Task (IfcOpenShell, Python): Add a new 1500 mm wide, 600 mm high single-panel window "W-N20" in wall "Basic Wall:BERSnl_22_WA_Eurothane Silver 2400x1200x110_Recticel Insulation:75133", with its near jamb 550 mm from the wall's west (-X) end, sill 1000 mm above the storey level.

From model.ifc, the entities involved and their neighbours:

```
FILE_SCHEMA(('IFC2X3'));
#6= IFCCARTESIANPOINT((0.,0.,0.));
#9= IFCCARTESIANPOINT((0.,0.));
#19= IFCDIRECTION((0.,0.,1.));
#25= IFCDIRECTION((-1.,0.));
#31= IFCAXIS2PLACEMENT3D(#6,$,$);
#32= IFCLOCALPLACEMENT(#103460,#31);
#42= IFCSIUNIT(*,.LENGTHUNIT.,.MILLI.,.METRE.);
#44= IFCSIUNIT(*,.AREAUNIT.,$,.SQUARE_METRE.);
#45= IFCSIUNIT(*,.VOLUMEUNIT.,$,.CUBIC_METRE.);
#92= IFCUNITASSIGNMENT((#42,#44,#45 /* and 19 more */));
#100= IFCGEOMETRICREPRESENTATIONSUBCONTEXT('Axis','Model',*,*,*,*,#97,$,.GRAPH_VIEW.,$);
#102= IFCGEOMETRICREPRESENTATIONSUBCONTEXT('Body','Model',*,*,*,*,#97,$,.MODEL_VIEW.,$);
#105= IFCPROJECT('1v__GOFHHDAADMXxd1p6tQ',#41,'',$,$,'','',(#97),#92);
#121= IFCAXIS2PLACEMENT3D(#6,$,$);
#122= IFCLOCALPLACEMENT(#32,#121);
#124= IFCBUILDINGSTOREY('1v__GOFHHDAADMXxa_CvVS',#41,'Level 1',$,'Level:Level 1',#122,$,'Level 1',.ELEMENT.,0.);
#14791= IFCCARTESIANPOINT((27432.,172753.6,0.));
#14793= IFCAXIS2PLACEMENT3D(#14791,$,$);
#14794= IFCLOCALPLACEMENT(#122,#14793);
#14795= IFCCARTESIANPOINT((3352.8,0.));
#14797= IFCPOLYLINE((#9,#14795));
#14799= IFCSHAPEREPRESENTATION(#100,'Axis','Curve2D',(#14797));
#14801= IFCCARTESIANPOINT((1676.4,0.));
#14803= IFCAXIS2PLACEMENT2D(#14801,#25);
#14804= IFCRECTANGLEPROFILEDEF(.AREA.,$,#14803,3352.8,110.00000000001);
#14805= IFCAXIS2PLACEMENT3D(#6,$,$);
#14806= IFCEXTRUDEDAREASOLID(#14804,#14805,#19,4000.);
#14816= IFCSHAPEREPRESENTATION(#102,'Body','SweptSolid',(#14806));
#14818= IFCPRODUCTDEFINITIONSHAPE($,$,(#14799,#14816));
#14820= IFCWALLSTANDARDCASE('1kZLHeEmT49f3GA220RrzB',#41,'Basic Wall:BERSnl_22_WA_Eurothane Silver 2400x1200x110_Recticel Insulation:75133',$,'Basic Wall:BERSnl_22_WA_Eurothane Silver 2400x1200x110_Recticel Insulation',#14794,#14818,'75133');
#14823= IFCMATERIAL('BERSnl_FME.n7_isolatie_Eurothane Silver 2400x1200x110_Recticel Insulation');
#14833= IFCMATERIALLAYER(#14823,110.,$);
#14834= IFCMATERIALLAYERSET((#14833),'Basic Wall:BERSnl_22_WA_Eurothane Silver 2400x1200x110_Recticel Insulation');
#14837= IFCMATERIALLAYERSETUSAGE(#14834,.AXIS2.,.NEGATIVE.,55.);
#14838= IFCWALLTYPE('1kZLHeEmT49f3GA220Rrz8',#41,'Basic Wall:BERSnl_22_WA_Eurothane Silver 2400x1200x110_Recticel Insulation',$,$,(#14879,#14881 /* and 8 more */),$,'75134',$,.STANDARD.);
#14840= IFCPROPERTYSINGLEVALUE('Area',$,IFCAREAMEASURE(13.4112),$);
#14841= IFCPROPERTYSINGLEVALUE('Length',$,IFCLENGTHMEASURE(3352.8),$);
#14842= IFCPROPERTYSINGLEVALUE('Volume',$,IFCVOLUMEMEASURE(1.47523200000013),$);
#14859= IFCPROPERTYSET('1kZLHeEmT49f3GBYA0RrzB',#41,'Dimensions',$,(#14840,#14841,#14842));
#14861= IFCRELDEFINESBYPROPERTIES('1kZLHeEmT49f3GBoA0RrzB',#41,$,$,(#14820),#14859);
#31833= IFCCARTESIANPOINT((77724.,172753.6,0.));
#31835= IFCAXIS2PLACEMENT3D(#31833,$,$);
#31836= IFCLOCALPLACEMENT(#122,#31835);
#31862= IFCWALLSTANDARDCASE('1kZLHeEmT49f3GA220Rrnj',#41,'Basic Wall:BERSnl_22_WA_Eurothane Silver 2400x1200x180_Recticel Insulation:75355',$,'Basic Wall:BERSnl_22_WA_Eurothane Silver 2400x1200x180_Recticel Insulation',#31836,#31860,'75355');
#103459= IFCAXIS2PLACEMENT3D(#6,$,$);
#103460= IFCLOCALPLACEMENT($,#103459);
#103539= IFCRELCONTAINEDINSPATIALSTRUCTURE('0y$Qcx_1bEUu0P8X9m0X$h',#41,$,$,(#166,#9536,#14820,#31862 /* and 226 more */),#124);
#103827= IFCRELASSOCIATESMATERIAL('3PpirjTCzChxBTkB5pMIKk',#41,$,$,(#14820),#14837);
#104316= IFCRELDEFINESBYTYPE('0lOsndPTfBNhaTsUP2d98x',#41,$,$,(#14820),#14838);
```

```python
import numpy as np
import ifcopenshell
import ifcopenshell.api.feature
import ifcopenshell.api.geometry
import ifcopenshell.api.pset
import ifcopenshell.api.root
import ifcopenshell.api.spatial
import ifcopenshell.api.type
import ifcopenshell.geom
import ifcopenshell.util.element
import ifcopenshell.util.placement
import ifcopenshell.util.representation
import ifcopenshell.util.shape
import ifcopenshell.util.unit

model = ifcopenshell.open("model.ifc")
unit_scale = ifcopenshell.util.unit.calculate_unit_scale(model)
area_scale = ifcopenshell.util.unit.calculate_unit_scale(model, "AREAUNIT")
volume_scale = ifcopenshell.util.unit.calculate_unit_scale(model, "VOLUMEUNIT")
settings = ifcopenshell.geom.settings()


def volume(element):
    """Net volume in cubic metres, openings subtracted."""
    shape = ifcopenshell.geom.create_shape(settings, element)
    return ifcopenshell.util.shape.get_volume(shape.geometry)


wall = model.by_guid("1kZLHeEmT49f3GA220RrzB")
storey = ifcopenshell.util.element.get_container(wall, ifc_class="IfcBuildingStorey")
context = ifcopenshell.util.representation.get_context(model, "Model", "Body", "MODEL_VIEW")
before = volume(wall)

width, height, from_end, sill = 1.5, 0.6, 0.55, 1  # metres

# The wall runs along its own X axis, and the end named is its -X end.
wall_shape = ifcopenshell.geom.create_shape(settings, wall)
x, y, z = ifcopenshell.util.shape.get_vertices(wall_shape.geometry).T
start = x.min() + from_end
face, thickness = float(y.min()), float(y.max() - y.min())
wall_matrix = ifcopenshell.util.placement.get_local_placement(wall.ObjectPlacement)
level = ifcopenshell.util.placement.get_local_placement(storey.ObjectPlacement)[2, 3]


def in_wall(x, y):
    """Placement at x, y metres in the wall's axes, at sill height."""
    matrix = wall_matrix.copy()
    matrix[:, 3] = wall_matrix @ np.array([x / unit_scale, y / unit_scale, 0.0, 1.0])
    matrix[2, 3] = level + sill / unit_scale
    return matrix


# Opening: a box that overshoots both wall faces by 50 mm.
opening = ifcopenshell.api.root.create_entity(model, ifc_class="IfcOpeningElement")
box = ifcopenshell.api.geometry.add_wall_representation(
    model, context=context, length=width, height=height, thickness=thickness + 0.1
)
ifcopenshell.api.geometry.assign_representation(model, product=opening, representation=box)
ifcopenshell.api.geometry.edit_object_placement(model, product=opening, matrix=in_wall(start, face - 0.05), is_si=False)
ifcopenshell.api.feature.add_feature(model, feature=opening, element=wall)

window = ifcopenshell.api.root.create_entity(model, ifc_class="IfcWindow", name="W-N20")
window.OverallWidth, window.OverallHeight = width / unit_scale, height / unit_scale
body = ifcopenshell.api.geometry.add_window_representation(
    model,
    context=context,
    overall_width=window.OverallWidth,
    overall_height=window.OverallHeight,
    partition_type="SINGLE_PANEL",
)
ifcopenshell.api.geometry.assign_representation(model, product=window, representation=body)
ifcopenshell.api.spatial.assign_container(model, products=[window], relating_structure=storey)
fills = ifcopenshell.api.feature.add_filling(model, opening=opening, element=window)
fills.OwnerHistory = window.OwnerHistory  # required in IFC2X3

# IFC2X3 keeps the operation on the window style.
style = ifcopenshell.api.root.create_entity(model, ifc_class="IfcWindowStyle", name="W-N20")
style.OperationType, style.ConstructionType = "SINGLE_PANEL", "NOTDEFINED"
style.ParameterTakesPrecedence = style.Sizeable = False
ifcopenshell.api.type.assign_type(model, related_objects=[window], relating_type=style)

# Centre the window in the wall's thickness.
ifcopenshell.api.geometry.edit_object_placement(model, product=window, matrix=in_wall(start, face), is_si=False)
window_shape = ifcopenshell.geom.create_shape(settings, window)
depth = ifcopenshell.util.shape.get_vertices(window_shape.geometry)[:, 1]
offset = face + thickness / 2 - (depth.min() + depth.max()) / 2
ifcopenshell.api.geometry.edit_object_placement(model, product=window, matrix=in_wall(start, offset), is_si=False)

after = volume(wall)

# Update the wall's stored quantities.
pset = model.by_id(ifcopenshell.util.element.get_pset(wall, "Dimensions", should_inherit=False)["id"])
ifcopenshell.api.pset.edit_pset(model, pset=pset, properties={
    "Area": model.create_entity("IfcAreaMeasure", after / thickness / area_scale),
    "Volume": model.create_entity("IfcVolumeMeasure", after / volume_scale),
})

print(f"wall volume {before:.3f} -> {after:.3f} m3")

model.write("model_v2.ifc")
```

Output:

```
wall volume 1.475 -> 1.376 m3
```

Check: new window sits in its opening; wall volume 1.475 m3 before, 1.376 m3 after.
